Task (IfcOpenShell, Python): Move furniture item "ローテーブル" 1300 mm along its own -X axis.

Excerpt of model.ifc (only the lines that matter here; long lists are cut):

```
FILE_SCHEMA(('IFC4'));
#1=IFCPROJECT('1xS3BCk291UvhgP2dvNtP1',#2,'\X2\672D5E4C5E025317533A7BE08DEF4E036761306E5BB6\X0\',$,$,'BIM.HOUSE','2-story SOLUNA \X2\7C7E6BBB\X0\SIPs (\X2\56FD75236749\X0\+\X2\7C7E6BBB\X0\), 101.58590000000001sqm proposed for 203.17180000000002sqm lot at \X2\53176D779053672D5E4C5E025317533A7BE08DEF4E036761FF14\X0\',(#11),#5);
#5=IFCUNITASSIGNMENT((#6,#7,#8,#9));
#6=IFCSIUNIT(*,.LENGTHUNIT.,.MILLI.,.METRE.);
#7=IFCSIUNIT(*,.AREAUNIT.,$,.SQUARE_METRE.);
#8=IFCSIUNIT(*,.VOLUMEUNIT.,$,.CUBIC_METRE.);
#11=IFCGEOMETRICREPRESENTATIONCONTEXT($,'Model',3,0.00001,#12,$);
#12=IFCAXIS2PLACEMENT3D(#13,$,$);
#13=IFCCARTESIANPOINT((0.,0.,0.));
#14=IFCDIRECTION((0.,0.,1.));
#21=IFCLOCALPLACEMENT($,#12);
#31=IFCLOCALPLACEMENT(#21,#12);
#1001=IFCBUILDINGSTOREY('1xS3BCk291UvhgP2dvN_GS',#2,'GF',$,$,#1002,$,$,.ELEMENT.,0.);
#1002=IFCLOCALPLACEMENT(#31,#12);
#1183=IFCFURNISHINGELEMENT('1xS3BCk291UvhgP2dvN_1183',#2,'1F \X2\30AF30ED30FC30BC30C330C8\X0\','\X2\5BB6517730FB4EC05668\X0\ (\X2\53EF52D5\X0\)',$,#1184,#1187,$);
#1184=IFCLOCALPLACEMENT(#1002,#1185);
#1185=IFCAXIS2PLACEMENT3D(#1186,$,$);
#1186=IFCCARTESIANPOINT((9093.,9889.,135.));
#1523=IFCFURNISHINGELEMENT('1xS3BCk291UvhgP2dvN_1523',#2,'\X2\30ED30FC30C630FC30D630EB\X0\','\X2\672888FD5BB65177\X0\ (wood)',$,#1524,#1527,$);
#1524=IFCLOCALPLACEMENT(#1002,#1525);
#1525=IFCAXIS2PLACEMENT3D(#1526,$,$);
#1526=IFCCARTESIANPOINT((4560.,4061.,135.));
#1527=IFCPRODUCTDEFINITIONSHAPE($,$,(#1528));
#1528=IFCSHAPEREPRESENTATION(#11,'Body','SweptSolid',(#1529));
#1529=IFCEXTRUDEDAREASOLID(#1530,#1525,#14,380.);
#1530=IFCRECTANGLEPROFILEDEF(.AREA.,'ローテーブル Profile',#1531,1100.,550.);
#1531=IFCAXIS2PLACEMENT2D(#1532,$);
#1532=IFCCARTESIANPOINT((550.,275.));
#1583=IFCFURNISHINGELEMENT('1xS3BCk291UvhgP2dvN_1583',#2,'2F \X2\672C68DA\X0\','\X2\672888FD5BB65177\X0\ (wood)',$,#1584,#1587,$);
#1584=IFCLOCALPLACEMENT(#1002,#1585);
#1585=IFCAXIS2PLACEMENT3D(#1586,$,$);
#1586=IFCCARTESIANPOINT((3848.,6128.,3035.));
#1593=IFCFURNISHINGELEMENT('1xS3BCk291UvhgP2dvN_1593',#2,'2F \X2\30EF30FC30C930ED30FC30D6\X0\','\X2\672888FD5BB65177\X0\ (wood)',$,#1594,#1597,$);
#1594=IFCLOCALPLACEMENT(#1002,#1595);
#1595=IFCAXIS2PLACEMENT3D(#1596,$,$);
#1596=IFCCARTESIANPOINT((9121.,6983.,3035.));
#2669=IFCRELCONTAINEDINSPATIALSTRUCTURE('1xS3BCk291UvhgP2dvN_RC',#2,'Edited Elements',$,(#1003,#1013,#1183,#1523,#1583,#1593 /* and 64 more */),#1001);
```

```python
import ifcopenshell
import ifcopenshell.api.geometry
import ifcopenshell.util.placement
import ifcopenshell.util.unit

model = ifcopenshell.open("model.ifc")
unit_scale = ifcopenshell.util.unit.calculate_unit_scale(model)

item = model.by_guid("1xS3BCk291UvhgP2dvN_1523")
matrix = ifcopenshell.util.placement.get_local_placement(item.ObjectPlacement)
matrix[:3, 3] -= matrix[:3, 0] * 1.3 / unit_scale
ifcopenshell.api.geometry.edit_object_placement(model, product=item, matrix=matrix, is_si=False)

print(ifcopenshell.util.placement.get_local_placement(item.ObjectPlacement).round(3) + 0.0)

model.write("model_rev.ifc")
```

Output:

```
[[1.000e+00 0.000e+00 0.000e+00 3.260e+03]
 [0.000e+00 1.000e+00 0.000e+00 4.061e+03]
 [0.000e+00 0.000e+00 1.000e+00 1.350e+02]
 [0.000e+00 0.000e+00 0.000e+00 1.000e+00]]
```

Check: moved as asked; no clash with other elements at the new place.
